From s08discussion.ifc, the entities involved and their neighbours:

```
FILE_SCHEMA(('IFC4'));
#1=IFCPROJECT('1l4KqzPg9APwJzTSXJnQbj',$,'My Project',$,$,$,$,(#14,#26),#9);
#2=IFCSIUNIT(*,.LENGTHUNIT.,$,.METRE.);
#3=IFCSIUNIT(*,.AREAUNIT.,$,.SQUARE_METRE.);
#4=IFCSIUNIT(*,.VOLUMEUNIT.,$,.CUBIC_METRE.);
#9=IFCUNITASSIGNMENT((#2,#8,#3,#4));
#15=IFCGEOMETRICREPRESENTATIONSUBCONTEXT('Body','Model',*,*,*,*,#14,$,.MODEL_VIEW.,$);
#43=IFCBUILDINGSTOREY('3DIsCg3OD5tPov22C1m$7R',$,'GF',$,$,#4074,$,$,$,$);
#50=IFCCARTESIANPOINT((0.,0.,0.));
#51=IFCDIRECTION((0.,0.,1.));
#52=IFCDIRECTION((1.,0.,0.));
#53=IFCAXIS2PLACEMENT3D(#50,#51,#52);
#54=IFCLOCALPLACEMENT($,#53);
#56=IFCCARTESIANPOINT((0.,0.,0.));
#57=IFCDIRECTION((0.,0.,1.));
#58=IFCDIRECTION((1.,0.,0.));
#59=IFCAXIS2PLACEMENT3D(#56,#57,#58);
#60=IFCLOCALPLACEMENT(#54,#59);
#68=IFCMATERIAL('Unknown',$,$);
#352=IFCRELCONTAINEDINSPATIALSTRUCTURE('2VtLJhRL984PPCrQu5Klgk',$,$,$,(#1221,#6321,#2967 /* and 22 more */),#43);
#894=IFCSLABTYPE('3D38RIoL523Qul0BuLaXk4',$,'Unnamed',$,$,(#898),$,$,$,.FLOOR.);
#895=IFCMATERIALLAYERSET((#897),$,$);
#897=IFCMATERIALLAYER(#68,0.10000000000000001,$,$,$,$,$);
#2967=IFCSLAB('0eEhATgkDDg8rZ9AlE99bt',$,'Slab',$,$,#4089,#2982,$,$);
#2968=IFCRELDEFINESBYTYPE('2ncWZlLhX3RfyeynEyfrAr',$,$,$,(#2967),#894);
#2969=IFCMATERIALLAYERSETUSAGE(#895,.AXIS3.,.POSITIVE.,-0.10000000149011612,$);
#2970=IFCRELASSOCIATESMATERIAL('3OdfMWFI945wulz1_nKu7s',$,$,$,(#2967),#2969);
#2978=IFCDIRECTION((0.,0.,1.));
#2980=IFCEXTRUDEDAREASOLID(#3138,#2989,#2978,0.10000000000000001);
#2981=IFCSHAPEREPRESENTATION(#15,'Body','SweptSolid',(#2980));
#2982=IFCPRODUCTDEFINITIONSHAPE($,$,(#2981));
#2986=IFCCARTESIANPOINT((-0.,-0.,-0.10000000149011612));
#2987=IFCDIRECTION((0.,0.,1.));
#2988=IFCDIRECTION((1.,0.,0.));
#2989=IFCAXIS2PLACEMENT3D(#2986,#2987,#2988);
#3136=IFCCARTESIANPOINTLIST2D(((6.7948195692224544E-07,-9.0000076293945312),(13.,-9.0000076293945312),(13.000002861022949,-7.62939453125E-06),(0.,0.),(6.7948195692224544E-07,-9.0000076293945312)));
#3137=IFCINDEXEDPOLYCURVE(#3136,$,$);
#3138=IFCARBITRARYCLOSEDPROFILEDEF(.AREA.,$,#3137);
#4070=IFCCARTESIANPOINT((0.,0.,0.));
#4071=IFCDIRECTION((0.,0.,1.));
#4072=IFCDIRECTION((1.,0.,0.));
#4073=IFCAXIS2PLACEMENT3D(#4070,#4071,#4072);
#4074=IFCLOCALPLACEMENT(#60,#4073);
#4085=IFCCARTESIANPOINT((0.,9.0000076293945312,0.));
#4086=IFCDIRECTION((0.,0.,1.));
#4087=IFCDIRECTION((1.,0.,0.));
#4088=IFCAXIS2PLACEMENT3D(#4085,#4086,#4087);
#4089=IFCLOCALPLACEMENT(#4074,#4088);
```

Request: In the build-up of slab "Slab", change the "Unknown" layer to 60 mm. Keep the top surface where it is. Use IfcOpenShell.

```python
import ifcopenshell
import ifcopenshell.util.element
import ifcopenshell.util.representation
import ifcopenshell.util.unit

model = ifcopenshell.open("s08discussion.ifc")
unit_scale = ifcopenshell.util.unit.calculate_unit_scale(model)

layer_set = model.by_id(895)
layer = next(l for l in layer_set.MaterialLayers if l.Material and l.Material.Name == "Unknown")
change = 0.06 / unit_scale - layer.LayerThickness
layer.LayerThickness += change

# Geometry does not follow the layer set by itself.
slabs = [e for e in ifcopenshell.util.element.get_elements_by_material(model, layer_set) if e.is_a("IfcSlab")]
for slab in sorted(slabs, key=lambda e: e.id()):
    body = ifcopenshell.util.representation.get_representation(slab, "Model", "Body")
    solid = body.Items[0]
    old_depth = solid.Depth
    solid.Depth += change
    # Extruded upwards: lower the start of the extrusion so the top stays.
    x, y, z = solid.Position.Location.Coordinates
    solid.Position.Location = model.createIfcCartesianPoint((x, y, z - change))
    print(slab.id(), f"{old_depth:g} -> {solid.Depth:g}")

# The layers are counted up from the underside, which has moved.
for usage in {ifcopenshell.util.element.get_material(slab) for slab in slabs}:
    usage.OffsetFromReferenceLine -= change

model.write("s08discussion_edited.ifc")
```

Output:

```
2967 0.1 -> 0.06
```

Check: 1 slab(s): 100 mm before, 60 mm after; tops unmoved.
